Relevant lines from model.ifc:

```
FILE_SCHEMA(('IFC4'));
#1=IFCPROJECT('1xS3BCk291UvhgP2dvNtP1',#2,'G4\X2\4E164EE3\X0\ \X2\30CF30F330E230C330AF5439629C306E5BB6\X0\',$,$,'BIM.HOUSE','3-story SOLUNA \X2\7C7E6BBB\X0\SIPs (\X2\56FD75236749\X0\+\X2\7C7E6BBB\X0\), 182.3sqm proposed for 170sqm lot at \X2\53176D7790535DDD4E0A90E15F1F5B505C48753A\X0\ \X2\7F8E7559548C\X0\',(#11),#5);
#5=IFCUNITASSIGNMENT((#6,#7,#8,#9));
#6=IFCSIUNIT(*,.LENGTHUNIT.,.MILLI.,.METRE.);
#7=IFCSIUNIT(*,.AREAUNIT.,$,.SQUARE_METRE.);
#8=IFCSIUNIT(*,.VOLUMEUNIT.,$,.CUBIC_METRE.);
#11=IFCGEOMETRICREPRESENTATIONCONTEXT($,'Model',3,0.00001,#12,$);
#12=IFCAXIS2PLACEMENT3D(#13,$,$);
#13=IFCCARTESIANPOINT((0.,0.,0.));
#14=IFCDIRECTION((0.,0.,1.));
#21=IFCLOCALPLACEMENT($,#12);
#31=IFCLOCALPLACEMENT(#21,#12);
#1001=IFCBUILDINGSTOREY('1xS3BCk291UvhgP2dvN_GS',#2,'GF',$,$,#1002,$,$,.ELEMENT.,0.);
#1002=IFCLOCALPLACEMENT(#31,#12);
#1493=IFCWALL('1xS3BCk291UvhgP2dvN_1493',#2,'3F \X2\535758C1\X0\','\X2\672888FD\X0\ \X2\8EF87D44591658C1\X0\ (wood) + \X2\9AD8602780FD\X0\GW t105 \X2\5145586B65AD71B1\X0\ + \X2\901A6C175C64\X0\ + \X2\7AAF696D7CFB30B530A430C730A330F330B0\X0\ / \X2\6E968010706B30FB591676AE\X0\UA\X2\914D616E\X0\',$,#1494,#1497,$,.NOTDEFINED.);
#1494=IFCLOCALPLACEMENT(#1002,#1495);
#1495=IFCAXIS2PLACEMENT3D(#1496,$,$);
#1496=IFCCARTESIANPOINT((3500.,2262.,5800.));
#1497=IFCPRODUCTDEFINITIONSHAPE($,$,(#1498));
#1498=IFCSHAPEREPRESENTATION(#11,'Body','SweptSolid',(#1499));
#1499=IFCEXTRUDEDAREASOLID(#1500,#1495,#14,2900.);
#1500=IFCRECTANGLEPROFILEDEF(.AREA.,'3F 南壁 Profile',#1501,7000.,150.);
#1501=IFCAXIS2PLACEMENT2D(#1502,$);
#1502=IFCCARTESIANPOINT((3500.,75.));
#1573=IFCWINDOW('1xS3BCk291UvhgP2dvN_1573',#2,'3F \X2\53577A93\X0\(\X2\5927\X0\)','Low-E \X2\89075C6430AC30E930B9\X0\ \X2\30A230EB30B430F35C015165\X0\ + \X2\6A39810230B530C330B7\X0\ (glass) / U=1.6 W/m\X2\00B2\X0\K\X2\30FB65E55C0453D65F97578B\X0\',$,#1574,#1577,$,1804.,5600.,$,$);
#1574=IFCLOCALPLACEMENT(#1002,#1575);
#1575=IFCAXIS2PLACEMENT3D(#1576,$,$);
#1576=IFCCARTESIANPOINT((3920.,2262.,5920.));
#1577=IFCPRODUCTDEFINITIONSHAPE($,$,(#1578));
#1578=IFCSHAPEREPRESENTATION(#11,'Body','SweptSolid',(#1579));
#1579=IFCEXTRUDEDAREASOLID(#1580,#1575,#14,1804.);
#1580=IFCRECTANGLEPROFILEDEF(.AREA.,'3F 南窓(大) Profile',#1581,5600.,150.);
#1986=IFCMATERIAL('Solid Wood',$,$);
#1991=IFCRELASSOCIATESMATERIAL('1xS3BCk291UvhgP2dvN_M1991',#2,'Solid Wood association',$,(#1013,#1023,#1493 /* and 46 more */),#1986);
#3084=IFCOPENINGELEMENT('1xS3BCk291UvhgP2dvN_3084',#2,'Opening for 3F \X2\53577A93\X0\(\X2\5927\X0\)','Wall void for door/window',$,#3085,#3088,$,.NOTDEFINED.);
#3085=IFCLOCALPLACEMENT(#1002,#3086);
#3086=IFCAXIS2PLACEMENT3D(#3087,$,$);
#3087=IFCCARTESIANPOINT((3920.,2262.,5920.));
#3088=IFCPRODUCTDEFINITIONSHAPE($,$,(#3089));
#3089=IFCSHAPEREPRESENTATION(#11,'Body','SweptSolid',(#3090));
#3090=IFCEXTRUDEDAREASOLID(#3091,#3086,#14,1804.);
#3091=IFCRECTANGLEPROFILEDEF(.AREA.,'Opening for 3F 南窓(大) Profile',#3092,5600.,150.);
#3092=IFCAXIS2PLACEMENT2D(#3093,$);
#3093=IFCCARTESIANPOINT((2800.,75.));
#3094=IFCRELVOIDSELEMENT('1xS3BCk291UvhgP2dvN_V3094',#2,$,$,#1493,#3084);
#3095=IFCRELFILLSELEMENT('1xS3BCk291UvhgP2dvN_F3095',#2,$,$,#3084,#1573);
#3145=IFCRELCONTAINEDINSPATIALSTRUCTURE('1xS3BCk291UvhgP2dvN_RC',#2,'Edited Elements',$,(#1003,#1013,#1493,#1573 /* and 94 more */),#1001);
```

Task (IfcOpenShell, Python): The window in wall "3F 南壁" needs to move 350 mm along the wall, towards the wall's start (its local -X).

```python
import ifcopenshell
import ifcopenshell.api.geometry
import ifcopenshell.util.placement
import ifcopenshell.util.unit

model = ifcopenshell.open("model.ifc")
unit_scale = ifcopenshell.util.unit.calculate_unit_scale(model)

window = model.by_guid("1xS3BCk291UvhgP2dvN_1573")
opening = window.FillsVoids[0].RelatingOpeningElement
wall = opening.VoidsElements[0].RelatingBuildingElement

wall_matrix = ifcopenshell.util.placement.get_local_placement(wall.ObjectPlacement)
shift = wall_matrix[:3, 0] * -0.35 / unit_scale
before = ifcopenshell.util.placement.get_local_placement(window.ObjectPlacement)[:3, 3].copy()

# The window is not placed relative to its opening, so move both.
for product in (opening, window):
    matrix = ifcopenshell.util.placement.get_local_placement(product.ObjectPlacement)
    matrix[:3, 3] += shift
    ifcopenshell.api.geometry.edit_object_placement(model, product=product, matrix=matrix, is_si=False)

after = ifcopenshell.util.placement.get_local_placement(window.ObjectPlacement)[:3, 3]
print("window moved by", (after - before).round(3) + 0.0)

model.write("model-out.ifc")
```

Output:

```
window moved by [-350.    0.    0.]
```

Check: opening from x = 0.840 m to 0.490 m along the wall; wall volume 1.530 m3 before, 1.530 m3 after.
